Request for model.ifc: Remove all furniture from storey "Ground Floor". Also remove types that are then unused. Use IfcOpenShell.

First a look at what the model holds.

```python
import ifcopenshell
import ifcopenshell.util.element

model = ifcopenshell.open("model.ifc")
print(model.schema)
storey = next(s for s in model.by_type("IfcBuildingStorey") if s.Name == "Ground Floor")
furniture = [e for e in ifcopenshell.util.element.get_decomposition(storey) if e.is_a("IfcFurnishingElement")]
seen = {}
for e in furniture:
    element_type = ifcopenshell.util.element.get_type(e)
    name = element_type.Name if element_type not in (None, e) else None
    seen[name] = seen.get(name, 0) + 1
for name, count in sorted(seen.items(), key=str):
    print(count, "x", name)
```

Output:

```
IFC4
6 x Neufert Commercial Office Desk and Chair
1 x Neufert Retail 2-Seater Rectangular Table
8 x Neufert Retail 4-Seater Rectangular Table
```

```python
import ifcopenshell
import ifcopenshell.api.root
import ifcopenshell.util.element

model = ifcopenshell.open("model.ifc")

storey = next(s for s in model.by_type("IfcBuildingStorey") if s.Name == "Ground Floor")
furniture = [e for e in ifcopenshell.util.element.get_decomposition(storey) if e.is_a("IfcFurnishingElement")]
types = {ifcopenshell.util.element.get_type(e) for e in furniture} - {None, *furniture}

for e in furniture:
    ifcopenshell.api.root.remove_product(model, product=e)
print(len(furniture), "removed")

unused = [t for t in types if not ifcopenshell.util.element.get_types(t)]
for t in unused:
    ifcopenshell.api.root.remove_product(model, product=t)
print(len(unused), "unused types removed")

model.write("model_v2.ifc")
```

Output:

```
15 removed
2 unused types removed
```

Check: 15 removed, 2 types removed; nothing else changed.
